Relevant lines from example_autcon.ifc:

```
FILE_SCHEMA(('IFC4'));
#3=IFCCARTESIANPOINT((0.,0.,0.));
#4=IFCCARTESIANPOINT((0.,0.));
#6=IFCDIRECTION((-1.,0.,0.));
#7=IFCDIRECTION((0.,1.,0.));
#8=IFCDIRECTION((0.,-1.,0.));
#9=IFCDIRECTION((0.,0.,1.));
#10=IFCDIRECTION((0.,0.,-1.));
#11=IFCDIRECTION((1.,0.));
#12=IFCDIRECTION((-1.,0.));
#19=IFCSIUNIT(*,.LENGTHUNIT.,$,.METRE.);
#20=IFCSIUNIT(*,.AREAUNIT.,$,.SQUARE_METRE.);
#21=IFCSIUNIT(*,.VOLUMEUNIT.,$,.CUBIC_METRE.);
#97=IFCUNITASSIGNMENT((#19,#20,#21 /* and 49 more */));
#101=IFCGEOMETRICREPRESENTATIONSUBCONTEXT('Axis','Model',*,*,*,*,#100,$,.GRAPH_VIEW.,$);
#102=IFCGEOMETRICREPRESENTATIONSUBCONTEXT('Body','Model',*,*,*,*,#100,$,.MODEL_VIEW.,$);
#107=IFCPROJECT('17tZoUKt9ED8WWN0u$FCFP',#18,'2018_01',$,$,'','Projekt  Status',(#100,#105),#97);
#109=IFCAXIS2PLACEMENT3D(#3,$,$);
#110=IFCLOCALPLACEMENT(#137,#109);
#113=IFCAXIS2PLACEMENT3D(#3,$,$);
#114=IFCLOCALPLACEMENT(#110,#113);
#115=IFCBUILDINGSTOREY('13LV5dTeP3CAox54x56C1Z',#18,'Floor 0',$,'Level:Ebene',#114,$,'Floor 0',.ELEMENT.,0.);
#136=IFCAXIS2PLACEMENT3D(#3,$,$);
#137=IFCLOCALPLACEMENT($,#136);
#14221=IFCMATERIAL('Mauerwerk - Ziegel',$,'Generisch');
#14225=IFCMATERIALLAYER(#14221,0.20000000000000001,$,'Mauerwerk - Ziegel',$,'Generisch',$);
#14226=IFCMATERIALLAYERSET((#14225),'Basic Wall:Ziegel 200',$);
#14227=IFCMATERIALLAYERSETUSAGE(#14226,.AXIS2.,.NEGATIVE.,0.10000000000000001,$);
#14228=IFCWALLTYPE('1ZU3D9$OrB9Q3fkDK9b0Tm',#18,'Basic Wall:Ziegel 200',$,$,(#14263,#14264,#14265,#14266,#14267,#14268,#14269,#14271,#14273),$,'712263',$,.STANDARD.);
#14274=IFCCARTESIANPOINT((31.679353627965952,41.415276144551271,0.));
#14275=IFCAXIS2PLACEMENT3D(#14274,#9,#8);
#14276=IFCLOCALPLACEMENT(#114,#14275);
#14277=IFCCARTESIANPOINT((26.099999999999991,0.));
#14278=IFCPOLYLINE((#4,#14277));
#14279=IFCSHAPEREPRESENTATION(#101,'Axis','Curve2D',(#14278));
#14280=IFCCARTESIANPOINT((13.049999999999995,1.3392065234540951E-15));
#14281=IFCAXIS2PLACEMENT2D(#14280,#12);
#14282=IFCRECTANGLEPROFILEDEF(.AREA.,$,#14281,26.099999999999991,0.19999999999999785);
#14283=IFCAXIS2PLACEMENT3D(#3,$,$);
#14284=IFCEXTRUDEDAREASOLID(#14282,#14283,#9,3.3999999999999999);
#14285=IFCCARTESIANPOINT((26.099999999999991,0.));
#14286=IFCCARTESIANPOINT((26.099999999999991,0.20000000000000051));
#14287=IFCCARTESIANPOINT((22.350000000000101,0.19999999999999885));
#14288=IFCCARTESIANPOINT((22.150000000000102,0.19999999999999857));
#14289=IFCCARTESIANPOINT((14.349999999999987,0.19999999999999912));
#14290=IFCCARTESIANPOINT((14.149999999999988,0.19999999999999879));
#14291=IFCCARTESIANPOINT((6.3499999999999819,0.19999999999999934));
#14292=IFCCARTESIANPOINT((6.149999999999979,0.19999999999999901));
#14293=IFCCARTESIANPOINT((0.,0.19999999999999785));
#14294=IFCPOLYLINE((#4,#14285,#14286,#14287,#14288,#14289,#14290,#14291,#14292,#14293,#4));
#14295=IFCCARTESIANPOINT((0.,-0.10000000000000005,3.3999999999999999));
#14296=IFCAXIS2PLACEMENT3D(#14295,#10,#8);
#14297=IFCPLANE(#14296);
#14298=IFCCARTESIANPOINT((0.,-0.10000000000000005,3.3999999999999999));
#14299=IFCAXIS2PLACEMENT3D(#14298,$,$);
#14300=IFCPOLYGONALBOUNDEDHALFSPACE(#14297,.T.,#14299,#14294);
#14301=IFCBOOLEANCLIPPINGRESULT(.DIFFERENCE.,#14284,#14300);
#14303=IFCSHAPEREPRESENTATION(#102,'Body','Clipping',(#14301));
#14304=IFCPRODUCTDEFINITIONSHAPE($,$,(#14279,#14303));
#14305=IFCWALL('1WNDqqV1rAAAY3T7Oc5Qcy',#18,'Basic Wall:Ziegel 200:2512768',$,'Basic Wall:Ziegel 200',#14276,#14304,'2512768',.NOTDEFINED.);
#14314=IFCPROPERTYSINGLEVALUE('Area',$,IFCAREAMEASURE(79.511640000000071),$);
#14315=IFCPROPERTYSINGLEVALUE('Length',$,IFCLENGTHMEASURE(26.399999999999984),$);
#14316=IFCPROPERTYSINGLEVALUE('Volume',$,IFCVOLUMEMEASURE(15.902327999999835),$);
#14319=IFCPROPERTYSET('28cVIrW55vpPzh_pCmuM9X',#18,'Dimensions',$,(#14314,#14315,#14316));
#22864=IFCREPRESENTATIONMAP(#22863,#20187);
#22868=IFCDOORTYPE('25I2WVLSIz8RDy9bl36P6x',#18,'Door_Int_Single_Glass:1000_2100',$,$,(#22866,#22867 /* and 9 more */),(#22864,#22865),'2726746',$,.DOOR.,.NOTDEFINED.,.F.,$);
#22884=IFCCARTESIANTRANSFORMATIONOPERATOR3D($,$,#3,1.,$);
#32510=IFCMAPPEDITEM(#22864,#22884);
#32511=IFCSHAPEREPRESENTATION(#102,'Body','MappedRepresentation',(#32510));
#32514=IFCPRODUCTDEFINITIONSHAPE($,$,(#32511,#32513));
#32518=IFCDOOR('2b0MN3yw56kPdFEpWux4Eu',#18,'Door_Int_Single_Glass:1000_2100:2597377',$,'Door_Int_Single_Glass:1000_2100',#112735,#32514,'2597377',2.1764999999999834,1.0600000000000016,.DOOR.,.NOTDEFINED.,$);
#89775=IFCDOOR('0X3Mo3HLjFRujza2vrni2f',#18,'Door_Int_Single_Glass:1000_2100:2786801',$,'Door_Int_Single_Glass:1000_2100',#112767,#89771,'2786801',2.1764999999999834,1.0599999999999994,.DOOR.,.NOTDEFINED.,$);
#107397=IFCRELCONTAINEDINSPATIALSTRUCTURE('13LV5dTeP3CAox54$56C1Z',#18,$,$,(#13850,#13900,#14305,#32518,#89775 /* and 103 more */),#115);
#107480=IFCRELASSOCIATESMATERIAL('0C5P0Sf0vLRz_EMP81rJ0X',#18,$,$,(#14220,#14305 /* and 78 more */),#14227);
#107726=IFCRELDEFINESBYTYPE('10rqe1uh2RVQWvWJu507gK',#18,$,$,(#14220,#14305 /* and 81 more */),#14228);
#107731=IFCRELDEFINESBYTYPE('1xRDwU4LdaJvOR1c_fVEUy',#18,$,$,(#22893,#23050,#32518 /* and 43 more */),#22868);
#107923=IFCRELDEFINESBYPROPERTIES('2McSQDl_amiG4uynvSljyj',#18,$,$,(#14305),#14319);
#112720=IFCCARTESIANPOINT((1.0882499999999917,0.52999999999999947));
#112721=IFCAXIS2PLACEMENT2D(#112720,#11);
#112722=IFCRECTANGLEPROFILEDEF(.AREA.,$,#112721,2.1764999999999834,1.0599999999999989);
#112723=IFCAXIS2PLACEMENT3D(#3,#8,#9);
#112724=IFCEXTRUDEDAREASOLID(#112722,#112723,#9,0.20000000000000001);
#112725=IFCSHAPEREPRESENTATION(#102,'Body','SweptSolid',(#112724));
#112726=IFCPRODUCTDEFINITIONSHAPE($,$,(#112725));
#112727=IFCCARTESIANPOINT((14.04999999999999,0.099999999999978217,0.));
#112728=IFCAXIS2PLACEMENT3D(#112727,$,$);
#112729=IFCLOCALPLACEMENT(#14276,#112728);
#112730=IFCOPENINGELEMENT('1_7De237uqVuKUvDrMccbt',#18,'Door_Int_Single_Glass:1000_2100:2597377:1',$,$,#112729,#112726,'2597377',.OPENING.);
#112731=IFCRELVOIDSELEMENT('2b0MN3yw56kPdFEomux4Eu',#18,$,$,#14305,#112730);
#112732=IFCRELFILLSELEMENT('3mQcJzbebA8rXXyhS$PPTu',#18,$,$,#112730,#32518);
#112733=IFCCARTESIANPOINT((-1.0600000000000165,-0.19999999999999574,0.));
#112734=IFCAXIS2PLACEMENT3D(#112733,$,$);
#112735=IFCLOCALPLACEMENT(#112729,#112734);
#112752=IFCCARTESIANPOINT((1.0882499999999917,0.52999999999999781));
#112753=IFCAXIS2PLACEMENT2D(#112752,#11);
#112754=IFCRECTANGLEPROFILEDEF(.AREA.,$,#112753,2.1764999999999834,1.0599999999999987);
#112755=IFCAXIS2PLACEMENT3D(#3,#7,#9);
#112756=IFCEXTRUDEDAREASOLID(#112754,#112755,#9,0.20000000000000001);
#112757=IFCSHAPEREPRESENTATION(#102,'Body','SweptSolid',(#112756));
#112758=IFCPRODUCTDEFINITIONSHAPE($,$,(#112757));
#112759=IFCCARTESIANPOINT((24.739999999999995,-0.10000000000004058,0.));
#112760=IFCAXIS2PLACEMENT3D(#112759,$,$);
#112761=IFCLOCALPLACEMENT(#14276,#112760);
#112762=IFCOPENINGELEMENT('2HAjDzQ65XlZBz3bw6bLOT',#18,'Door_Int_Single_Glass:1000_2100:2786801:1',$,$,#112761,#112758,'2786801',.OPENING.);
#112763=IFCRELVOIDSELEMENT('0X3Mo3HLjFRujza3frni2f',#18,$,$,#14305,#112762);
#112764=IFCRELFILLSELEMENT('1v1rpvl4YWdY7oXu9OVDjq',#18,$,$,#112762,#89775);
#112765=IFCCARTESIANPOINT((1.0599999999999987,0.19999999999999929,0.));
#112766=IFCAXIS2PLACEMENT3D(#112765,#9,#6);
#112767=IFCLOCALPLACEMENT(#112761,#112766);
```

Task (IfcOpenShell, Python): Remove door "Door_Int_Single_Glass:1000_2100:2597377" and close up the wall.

```python
import ifcopenshell
import ifcopenshell.api.feature
import ifcopenshell.api.pset
import ifcopenshell.api.root
import ifcopenshell.geom
import ifcopenshell.util.element
import ifcopenshell.util.shape
import ifcopenshell.util.unit

model = ifcopenshell.open("example_autcon.ifc")
area_scale = ifcopenshell.util.unit.calculate_unit_scale(model, "AREAUNIT")
volume_scale = ifcopenshell.util.unit.calculate_unit_scale(model, "VOLUMEUNIT")
settings = ifcopenshell.geom.settings()


def volume(element):
    """Net volume in cubic metres, openings subtracted."""
    shape = ifcopenshell.geom.create_shape(settings, element)
    return ifcopenshell.util.shape.get_volume(shape.geometry)


door = model.by_guid("2b0MN3yw56kPdFEpWux4Eu")
opening = door.FillsVoids[0].RelatingOpeningElement
wall = opening.VoidsElements[0].RelatingBuildingElement
before = volume(wall)

ifcopenshell.api.root.remove_product(model, product=door)
ifcopenshell.api.feature.remove_feature(model, feature=opening)

after = volume(wall)
thickness = 0.2  # wall thickness in metres

# Update the wall's stored quantities.
pset = model.by_id(ifcopenshell.util.element.get_pset(wall, "Dimensions", should_inherit=False)["id"])
ifcopenshell.api.pset.edit_pset(model, pset=pset, properties={
    "Area": model.create_entity("IfcAreaMeasure", after / thickness / area_scale),
    "Volume": model.create_entity("IfcVolumeMeasure", after / volume_scale),
})

print(f"wall volume {before:.3f} -> {after:.3f} m3")

model.write("example_autcon-out.ifc")
```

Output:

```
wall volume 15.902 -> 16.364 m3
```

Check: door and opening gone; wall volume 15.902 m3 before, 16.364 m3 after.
